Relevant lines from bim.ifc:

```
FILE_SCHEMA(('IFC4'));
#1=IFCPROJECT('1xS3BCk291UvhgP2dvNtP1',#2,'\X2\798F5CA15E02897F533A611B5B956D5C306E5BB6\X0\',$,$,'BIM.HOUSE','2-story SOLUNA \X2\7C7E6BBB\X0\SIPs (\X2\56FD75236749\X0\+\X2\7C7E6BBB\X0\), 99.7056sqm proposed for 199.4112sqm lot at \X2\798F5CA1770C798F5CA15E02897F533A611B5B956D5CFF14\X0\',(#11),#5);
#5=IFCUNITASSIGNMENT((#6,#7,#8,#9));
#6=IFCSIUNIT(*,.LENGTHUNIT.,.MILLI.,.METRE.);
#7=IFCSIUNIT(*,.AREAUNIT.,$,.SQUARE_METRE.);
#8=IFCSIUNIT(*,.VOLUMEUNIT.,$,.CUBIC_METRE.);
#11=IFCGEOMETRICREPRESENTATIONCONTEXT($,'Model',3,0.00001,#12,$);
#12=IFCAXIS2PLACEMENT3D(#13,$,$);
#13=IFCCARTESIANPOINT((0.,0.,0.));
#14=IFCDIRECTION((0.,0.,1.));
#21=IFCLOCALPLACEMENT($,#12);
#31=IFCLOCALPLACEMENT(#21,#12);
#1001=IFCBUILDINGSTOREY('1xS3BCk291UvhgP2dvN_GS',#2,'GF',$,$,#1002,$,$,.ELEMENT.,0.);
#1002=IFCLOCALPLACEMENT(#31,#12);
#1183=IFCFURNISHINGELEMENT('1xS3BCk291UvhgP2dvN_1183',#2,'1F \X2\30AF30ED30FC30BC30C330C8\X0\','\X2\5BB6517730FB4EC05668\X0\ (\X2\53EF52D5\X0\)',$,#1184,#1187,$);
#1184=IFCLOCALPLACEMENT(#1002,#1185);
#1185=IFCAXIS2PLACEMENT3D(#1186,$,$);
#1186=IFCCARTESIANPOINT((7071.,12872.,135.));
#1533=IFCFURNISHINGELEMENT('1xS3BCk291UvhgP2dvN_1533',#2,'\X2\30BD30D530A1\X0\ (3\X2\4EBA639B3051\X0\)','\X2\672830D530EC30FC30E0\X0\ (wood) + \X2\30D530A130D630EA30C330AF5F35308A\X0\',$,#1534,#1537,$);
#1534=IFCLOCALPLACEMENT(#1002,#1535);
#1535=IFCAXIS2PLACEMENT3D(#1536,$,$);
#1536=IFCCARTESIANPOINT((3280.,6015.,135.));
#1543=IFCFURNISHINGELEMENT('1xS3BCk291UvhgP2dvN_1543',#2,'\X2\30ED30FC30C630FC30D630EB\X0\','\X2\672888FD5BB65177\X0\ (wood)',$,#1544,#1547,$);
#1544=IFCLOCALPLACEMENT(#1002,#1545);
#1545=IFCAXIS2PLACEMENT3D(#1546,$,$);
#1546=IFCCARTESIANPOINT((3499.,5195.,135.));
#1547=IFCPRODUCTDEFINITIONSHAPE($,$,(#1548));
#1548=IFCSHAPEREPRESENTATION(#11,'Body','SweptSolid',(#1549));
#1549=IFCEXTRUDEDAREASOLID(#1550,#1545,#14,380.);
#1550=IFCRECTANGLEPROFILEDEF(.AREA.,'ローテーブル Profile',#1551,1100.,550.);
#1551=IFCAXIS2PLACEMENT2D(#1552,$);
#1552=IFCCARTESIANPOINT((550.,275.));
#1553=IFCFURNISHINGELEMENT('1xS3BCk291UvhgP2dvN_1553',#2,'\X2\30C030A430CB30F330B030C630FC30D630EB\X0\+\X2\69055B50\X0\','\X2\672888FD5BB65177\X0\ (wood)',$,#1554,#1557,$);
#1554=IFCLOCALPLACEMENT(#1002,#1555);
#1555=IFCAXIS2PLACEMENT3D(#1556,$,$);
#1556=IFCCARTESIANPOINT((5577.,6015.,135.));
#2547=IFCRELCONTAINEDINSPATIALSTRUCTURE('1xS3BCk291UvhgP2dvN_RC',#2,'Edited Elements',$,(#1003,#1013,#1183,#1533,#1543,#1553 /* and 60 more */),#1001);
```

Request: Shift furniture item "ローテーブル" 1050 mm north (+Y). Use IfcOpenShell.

```python
import ifcopenshell
import ifcopenshell.api.geometry
import ifcopenshell.util.placement
import ifcopenshell.util.unit

model = ifcopenshell.open("bim.ifc")
unit_scale = ifcopenshell.util.unit.calculate_unit_scale(model)

item = model.by_guid("1xS3BCk291UvhgP2dvN_1543")
matrix = ifcopenshell.util.placement.get_local_placement(item.ObjectPlacement)
matrix[1, 3] += 1.05 / unit_scale
ifcopenshell.api.geometry.edit_object_placement(model, product=item, matrix=matrix, is_si=False)

print(ifcopenshell.util.placement.get_local_placement(item.ObjectPlacement).round(3) + 0.0)

model.write("bim_rev.ifc")
```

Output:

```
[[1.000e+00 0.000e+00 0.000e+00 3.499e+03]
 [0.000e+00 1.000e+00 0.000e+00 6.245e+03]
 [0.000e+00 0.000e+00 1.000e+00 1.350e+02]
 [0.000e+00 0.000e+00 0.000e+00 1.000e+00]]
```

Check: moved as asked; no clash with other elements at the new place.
